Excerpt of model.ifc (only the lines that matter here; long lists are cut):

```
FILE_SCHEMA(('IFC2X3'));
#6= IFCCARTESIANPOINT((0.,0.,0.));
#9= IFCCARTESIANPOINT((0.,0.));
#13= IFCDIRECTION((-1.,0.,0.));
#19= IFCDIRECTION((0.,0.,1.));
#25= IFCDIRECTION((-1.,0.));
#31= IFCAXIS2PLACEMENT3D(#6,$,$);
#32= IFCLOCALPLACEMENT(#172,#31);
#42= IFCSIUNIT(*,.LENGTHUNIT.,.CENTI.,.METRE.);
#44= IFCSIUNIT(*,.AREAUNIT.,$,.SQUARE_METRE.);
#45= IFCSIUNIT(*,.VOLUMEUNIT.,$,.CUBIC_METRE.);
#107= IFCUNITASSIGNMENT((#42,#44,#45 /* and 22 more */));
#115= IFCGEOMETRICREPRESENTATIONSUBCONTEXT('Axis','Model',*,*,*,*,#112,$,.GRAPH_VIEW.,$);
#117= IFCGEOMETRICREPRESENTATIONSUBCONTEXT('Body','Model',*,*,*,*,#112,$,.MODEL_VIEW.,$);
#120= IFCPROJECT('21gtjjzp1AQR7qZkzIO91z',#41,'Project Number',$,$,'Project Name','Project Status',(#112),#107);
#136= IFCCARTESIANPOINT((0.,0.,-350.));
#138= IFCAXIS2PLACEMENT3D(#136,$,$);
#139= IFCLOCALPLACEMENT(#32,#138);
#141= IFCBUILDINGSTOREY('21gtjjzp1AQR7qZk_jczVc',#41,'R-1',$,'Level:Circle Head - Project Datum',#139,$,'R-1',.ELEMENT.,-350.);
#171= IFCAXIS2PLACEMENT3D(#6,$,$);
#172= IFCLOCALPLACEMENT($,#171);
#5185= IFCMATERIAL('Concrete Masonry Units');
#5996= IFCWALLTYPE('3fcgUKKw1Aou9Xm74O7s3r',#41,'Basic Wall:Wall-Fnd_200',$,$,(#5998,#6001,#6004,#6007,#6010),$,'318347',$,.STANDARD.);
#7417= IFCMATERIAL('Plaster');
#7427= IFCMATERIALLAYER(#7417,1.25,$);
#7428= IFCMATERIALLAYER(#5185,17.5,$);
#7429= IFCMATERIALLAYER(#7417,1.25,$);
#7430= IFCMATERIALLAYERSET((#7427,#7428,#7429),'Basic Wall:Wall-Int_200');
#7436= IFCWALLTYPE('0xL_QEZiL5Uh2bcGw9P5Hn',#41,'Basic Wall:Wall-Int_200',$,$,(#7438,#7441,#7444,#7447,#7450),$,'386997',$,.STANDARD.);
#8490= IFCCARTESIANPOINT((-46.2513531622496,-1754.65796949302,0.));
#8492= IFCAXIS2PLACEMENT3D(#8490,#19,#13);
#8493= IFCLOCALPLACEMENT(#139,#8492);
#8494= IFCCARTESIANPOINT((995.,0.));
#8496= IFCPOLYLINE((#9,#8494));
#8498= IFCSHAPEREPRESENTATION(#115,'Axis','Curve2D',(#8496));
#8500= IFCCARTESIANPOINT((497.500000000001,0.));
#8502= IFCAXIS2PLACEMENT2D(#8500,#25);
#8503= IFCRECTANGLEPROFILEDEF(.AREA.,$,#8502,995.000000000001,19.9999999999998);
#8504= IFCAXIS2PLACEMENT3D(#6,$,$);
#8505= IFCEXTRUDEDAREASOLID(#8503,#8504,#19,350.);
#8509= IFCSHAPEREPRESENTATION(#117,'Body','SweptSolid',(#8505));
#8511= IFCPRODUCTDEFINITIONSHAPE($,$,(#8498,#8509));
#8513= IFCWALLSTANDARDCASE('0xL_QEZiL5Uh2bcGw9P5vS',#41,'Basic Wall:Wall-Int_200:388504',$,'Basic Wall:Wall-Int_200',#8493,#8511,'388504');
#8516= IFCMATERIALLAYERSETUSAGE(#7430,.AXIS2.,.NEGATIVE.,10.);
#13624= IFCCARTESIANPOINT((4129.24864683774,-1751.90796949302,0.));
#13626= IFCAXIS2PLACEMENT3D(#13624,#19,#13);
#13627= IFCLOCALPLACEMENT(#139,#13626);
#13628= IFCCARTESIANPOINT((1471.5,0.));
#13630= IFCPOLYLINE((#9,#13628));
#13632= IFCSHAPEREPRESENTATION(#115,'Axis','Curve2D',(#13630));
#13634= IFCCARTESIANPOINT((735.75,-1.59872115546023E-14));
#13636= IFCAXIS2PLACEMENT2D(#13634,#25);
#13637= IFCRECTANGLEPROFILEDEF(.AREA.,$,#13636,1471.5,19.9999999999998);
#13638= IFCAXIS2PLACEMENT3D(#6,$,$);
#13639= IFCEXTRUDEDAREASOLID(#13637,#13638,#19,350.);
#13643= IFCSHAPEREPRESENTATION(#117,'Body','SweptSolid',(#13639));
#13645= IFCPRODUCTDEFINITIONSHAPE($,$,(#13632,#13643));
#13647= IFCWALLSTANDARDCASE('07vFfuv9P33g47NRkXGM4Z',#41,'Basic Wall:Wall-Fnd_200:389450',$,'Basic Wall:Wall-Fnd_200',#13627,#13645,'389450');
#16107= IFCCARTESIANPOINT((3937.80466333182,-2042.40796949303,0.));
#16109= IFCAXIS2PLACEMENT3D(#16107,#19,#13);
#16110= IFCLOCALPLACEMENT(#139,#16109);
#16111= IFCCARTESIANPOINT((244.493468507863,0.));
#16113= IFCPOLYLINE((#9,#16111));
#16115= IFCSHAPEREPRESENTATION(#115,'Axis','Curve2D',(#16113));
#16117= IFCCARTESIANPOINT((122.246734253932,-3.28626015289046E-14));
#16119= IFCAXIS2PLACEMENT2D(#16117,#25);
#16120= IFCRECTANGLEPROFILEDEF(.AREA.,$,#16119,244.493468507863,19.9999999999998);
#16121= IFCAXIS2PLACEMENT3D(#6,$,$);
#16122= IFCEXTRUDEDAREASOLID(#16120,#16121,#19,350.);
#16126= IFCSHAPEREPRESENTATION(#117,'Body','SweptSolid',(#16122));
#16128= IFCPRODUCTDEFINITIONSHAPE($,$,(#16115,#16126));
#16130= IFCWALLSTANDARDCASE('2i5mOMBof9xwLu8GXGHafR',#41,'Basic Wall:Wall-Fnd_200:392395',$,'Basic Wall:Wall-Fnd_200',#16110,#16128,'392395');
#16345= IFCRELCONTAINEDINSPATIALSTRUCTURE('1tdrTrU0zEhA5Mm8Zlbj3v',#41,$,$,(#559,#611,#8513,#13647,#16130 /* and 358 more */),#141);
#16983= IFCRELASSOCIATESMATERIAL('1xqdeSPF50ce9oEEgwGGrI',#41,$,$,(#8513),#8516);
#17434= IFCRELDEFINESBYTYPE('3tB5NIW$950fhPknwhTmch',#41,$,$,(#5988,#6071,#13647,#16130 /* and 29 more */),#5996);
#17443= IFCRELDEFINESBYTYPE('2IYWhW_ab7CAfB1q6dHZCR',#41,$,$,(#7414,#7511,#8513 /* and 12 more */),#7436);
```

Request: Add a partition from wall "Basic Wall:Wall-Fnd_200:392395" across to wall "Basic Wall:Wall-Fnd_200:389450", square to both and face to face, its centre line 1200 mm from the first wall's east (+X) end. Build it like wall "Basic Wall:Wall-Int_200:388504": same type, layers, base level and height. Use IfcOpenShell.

```python
import numpy as np
import ifcopenshell
import ifcopenshell.api.geometry
import ifcopenshell.api.material
import ifcopenshell.api.pset
import ifcopenshell.api.root
import ifcopenshell.api.spatial
import ifcopenshell.api.type
import ifcopenshell.geom
import ifcopenshell.util.element
import ifcopenshell.util.placement
import ifcopenshell.util.representation
import ifcopenshell.util.shape
import ifcopenshell.util.unit

model = ifcopenshell.open("model.ifc")
unit_scale = ifcopenshell.util.unit.calculate_unit_scale(model)
settings = ifcopenshell.geom.settings()
settings.set("use-world-coords", True)

start_wall = model.by_guid("2i5mOMBof9xwLu8GXGHafR")
end_wall = model.by_guid("07vFfuv9P33g47NRkXGM4Z")
like = model.by_guid("0xL_QEZiL5Uh2bcGw9P5vS")
matrix = ifcopenshell.util.placement.get_local_placement(start_wall.ObjectPlacement)
matrix[:3, 3] *= unit_scale


def extent(element):
    """Bounding box in the first wall's axes, in metres."""
    shape = ifcopenshell.geom.create_shape(settings, element)
    points = (ifcopenshell.util.shape.get_vertices(shape.geometry) - matrix[:3, 3]) @ matrix[:3, :3]
    return points.min(axis=0), points.max(axis=0)


y_start = extent(start_wall)[0][1]
y_end = extent(end_wall)[1][1]
like_min, like_max = extent(like)
length, height = float(abs(y_end - y_start)), float(like_max[2] - like_min[2])
layer_set = ifcopenshell.util.element.get_material(like, should_skip_usage=True)
thickness = sum(layer.LayerThickness for layer in layer_set.MaterialLayers) * unit_scale

wall = ifcopenshell.api.root.create_entity(model, ifc_class="IfcWallStandardCase", name="New partition")
storey = ifcopenshell.util.element.get_container(like)
ifcopenshell.api.spatial.assign_container(model, products=[wall], relating_structure=storey)
ifcopenshell.api.type.assign_type(
    model, related_objects=[wall], relating_type=ifcopenshell.util.element.get_type(like), should_map_representations=False
)
rel = ifcopenshell.api.material.assign_material(
    model, products=[wall], type="IfcMaterialLayerSetUsage", material=layer_set
)
rel.RelatingMaterial.OffsetFromReferenceLine = -thickness / 2 / unit_scale
pset = ifcopenshell.api.pset.add_pset(model, product=wall, name="Pset_WallCommon")
ifcopenshell.api.pset.edit_pset(model, pset=pset, properties={"IsExternal": False, "LoadBearing": False})

# The axis runs down the middle of the wall.
axis = ifcopenshell.api.geometry.add_axis_representation(
    model, context=ifcopenshell.util.representation.get_context(model, "Model", "Axis"), axis=[(0.0, 0.0), (length, 0.0)]
)
body = ifcopenshell.api.geometry.add_wall_representation(
    model,
    context=ifcopenshell.util.representation.get_context(model, "Model", "Body", "MODEL_VIEW"),
    length=length,
    height=height,
    thickness=thickness,
    offset=-thickness / 2,
)
for representation in (axis, body):
    ifcopenshell.api.geometry.assign_representation(model, product=wall, representation=representation)

placement = matrix @ ifcopenshell.util.placement.rotation(-90, "Z")
placement[:, 3] = matrix @ np.array([extent(start_wall)[0][0] + 1.2, y_start, like_min[2], 1.0])
ifcopenshell.api.geometry.edit_object_placement(model, product=wall, matrix=placement)

print(f"partition {length:.3f} m long, {height:.3f} m high, {thickness:.3f} m thick")

model.write("model_rev.ifc")
```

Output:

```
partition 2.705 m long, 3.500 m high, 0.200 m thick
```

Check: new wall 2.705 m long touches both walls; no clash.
